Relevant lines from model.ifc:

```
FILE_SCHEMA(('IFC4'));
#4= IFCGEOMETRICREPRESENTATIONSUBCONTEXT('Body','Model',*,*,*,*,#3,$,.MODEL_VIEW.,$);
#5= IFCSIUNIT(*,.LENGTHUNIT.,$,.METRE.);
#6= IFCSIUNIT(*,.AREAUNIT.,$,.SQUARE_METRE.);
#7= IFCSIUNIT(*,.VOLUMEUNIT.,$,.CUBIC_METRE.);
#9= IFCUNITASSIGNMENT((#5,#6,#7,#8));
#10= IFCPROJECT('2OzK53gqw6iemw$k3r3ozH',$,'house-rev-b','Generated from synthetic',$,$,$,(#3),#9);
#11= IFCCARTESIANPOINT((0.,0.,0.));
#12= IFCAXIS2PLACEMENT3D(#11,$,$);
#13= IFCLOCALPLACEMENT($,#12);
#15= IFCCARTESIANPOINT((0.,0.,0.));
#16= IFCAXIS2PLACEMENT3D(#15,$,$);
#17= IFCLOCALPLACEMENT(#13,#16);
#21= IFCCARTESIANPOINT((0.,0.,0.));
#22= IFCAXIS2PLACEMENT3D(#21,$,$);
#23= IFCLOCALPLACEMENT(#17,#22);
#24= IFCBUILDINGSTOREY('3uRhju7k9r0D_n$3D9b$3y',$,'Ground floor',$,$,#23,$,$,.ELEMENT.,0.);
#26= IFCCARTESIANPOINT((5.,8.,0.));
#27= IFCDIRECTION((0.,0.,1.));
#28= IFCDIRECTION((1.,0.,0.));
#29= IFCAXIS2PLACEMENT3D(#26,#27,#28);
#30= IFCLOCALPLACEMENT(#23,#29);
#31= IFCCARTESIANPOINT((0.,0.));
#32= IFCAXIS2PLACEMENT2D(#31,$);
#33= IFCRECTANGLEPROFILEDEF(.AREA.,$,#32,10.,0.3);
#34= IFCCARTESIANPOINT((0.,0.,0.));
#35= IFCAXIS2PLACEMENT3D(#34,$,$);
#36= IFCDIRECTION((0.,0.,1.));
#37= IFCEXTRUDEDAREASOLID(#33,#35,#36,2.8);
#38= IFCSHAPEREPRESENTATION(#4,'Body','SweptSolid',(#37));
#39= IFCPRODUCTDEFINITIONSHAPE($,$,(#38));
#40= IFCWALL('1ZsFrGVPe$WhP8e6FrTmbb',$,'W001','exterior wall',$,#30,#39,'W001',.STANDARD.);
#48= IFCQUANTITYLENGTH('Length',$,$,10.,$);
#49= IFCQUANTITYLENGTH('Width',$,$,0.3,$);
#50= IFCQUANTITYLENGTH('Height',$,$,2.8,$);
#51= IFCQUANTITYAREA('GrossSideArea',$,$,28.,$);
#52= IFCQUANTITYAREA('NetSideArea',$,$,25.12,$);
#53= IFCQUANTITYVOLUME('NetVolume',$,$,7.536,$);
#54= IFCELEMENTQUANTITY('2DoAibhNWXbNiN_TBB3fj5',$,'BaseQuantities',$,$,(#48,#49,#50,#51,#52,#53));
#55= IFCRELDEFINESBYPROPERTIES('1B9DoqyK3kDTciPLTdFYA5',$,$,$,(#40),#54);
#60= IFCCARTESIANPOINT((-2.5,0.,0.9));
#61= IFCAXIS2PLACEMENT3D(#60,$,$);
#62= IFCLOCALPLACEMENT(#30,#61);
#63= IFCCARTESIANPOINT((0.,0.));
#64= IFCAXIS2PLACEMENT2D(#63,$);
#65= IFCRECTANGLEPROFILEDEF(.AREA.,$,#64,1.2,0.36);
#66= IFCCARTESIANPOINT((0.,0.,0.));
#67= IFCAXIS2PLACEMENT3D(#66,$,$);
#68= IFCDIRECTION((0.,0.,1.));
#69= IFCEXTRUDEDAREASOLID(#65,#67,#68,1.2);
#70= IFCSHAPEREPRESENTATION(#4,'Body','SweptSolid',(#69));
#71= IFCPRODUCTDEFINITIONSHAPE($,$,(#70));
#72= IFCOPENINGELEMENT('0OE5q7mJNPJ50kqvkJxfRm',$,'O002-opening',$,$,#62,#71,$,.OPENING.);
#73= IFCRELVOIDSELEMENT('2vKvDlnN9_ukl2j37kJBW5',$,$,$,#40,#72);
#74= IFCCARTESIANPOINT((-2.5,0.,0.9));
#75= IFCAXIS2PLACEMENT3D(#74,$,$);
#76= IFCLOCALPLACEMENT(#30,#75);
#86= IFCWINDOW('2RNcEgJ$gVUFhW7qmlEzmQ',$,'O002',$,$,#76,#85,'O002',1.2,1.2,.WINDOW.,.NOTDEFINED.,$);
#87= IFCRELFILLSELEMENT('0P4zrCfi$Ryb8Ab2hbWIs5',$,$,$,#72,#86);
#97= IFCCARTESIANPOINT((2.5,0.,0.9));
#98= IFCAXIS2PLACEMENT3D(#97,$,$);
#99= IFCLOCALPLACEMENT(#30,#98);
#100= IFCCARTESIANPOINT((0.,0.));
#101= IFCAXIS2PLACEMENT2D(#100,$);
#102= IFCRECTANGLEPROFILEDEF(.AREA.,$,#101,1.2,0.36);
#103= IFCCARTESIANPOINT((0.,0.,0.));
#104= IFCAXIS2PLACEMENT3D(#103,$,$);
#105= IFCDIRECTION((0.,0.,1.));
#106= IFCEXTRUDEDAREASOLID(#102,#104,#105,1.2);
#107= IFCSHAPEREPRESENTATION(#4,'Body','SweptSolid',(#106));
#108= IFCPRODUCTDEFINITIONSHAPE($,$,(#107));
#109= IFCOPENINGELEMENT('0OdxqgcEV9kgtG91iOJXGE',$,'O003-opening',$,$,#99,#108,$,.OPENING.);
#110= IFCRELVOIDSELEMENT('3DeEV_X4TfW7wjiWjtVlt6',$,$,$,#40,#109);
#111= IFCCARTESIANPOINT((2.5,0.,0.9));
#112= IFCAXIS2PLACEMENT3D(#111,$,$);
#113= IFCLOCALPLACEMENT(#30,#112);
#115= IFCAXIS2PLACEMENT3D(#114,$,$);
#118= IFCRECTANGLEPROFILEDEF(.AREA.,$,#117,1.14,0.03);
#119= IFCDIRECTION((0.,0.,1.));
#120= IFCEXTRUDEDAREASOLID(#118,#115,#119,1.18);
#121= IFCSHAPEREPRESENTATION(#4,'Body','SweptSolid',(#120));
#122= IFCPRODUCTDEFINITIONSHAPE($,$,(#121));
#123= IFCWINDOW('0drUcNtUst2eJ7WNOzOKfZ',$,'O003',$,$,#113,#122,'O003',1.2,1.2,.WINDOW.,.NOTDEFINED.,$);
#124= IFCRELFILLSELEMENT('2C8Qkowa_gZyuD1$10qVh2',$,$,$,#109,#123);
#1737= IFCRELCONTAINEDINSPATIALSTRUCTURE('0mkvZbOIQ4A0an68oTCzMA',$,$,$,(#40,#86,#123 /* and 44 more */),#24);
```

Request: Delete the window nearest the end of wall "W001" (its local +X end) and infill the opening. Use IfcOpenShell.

```python
import ifcopenshell
import ifcopenshell.api.feature
import ifcopenshell.api.pset
import ifcopenshell.api.root
import ifcopenshell.geom
import ifcopenshell.util.element
import ifcopenshell.util.shape
import ifcopenshell.util.unit

model = ifcopenshell.open("model.ifc")
area_scale = ifcopenshell.util.unit.calculate_unit_scale(model, "AREAUNIT")
volume_scale = ifcopenshell.util.unit.calculate_unit_scale(model, "VOLUMEUNIT")
settings = ifcopenshell.geom.settings()


def volume(element):
    """Net volume in cubic metres, openings subtracted."""
    shape = ifcopenshell.geom.create_shape(settings, element)
    return ifcopenshell.util.shape.get_volume(shape.geometry)


window = model.by_guid("0drUcNtUst2eJ7WNOzOKfZ")
opening = window.FillsVoids[0].RelatingOpeningElement
wall = opening.VoidsElements[0].RelatingBuildingElement
before = volume(wall)

ifcopenshell.api.root.remove_product(model, product=window)
ifcopenshell.api.feature.remove_feature(model, feature=opening)

after = volume(wall)
thickness = 0.3  # wall thickness in metres

# Update the wall's stored quantities.
qto = model.by_id(ifcopenshell.util.element.get_pset(wall, "BaseQuantities", should_inherit=False)["id"])
ifcopenshell.api.pset.edit_qto(model, qto=qto, properties={
    "NetSideArea": after / thickness / area_scale,
    "NetVolume": after / volume_scale,
})

print(f"wall volume {before:.3f} -> {after:.3f} m3")

model.write("model_edited.ifc")
```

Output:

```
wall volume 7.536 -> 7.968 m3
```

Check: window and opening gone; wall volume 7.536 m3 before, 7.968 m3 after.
